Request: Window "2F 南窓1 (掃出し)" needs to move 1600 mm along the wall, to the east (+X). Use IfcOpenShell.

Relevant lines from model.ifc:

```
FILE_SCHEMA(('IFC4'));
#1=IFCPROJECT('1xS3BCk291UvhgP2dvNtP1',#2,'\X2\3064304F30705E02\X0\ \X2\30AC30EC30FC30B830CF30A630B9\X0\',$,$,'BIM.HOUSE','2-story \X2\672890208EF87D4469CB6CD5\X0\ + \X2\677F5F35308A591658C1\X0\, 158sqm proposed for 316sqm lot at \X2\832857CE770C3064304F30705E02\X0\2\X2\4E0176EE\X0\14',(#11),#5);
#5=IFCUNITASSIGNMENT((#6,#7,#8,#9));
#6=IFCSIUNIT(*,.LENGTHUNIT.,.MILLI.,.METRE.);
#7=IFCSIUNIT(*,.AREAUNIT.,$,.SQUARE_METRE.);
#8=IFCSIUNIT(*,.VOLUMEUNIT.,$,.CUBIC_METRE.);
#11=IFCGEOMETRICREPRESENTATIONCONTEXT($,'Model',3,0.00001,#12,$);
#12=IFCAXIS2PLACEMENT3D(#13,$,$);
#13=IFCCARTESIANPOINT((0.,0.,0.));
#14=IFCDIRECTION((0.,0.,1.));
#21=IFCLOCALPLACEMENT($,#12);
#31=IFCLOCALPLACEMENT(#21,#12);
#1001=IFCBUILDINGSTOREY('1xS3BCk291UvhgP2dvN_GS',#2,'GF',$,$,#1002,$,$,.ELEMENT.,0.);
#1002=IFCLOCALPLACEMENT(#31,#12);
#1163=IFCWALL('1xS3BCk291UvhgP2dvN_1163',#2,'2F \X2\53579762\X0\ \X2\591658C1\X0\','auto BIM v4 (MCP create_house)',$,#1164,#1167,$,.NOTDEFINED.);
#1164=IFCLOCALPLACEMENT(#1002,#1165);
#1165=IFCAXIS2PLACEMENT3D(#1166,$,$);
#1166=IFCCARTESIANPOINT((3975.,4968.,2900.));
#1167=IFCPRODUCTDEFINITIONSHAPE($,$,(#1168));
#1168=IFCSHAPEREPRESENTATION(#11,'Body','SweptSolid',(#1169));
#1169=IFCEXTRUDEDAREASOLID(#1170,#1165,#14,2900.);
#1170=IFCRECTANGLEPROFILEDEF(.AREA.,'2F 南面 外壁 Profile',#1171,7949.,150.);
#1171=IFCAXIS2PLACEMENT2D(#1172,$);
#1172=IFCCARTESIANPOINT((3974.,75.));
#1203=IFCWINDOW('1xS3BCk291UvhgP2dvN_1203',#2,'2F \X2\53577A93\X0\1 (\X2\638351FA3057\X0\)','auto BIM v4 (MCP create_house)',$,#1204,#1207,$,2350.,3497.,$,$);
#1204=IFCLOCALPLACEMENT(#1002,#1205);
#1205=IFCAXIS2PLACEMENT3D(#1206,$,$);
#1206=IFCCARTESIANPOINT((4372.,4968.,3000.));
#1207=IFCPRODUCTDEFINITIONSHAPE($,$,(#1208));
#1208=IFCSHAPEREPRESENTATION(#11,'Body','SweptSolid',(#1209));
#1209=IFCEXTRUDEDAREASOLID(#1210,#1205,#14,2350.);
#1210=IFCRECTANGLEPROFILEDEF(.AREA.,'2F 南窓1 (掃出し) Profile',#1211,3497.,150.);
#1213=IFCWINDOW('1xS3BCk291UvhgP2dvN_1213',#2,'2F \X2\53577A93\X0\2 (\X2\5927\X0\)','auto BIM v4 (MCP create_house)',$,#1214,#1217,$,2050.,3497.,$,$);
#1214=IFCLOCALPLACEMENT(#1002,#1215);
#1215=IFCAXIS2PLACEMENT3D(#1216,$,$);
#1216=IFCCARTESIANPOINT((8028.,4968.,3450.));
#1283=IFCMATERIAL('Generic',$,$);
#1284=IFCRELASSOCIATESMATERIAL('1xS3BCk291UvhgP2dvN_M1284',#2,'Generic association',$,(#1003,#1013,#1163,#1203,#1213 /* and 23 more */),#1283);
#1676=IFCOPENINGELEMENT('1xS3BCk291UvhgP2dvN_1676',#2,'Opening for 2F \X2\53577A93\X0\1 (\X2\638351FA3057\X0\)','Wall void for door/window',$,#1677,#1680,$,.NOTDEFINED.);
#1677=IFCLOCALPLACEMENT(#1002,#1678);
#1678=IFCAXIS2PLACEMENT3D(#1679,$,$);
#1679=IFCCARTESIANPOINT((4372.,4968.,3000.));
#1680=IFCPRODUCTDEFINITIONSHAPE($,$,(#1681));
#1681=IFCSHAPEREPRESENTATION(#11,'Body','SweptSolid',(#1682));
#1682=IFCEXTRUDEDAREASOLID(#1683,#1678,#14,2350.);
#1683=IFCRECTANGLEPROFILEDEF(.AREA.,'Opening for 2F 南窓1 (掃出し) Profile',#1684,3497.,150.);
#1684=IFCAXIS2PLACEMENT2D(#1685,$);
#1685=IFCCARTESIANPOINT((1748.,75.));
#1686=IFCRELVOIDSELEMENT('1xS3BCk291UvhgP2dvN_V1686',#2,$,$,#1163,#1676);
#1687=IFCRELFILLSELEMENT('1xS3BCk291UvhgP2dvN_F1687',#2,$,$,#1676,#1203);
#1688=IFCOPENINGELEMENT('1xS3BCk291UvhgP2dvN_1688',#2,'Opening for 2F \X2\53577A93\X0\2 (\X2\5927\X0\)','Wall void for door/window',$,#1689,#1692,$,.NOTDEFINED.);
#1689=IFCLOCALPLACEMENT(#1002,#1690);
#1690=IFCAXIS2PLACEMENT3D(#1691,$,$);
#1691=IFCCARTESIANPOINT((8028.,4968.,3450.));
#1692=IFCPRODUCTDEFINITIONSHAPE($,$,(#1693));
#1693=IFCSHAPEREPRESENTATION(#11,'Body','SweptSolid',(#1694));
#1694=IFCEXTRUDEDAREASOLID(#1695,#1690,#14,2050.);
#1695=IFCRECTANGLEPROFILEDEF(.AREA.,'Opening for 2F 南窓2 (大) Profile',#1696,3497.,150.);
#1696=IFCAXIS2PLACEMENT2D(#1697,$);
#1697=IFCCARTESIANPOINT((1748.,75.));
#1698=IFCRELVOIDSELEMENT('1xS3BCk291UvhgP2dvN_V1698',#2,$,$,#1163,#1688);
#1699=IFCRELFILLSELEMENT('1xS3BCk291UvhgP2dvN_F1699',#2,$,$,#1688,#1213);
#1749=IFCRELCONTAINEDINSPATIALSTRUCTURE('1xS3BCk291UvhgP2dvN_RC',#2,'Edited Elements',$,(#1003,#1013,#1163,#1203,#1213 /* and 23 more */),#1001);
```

```python
import ifcopenshell
import ifcopenshell.api.geometry
import ifcopenshell.util.placement
import ifcopenshell.util.unit

model = ifcopenshell.open("model.ifc")
unit_scale = ifcopenshell.util.unit.calculate_unit_scale(model)

window = model.by_id(1203)
opening = window.FillsVoids[0].RelatingOpeningElement
wall = opening.VoidsElements[0].RelatingBuildingElement

wall_matrix = ifcopenshell.util.placement.get_local_placement(wall.ObjectPlacement)
shift = wall_matrix[:3, 0] * 1.6 / unit_scale
before = ifcopenshell.util.placement.get_local_placement(window.ObjectPlacement)[:3, 3].copy()

# The window is not placed relative to its opening, so move both.
for product in (opening, window):
    matrix = ifcopenshell.util.placement.get_local_placement(product.ObjectPlacement)
    matrix[:3, 3] += shift
    ifcopenshell.api.geometry.edit_object_placement(model, product=product, matrix=matrix, is_si=False)

after = ifcopenshell.util.placement.get_local_placement(window.ObjectPlacement)[:3, 3]
print("window moved by", (after - before).round(3) + 0.0)

model.write("model_v2.ifc")
```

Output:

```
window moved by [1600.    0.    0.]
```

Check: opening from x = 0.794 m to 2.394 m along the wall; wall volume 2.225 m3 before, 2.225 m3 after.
